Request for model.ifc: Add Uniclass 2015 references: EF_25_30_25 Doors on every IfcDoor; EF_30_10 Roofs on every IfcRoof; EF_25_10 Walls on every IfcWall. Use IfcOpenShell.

First a look at what the model holds.

```python
import ifcopenshell

model = ifcopenshell.open("model.ifc")
print(model.schema)
print("classifications:", [c.Name for c in model.by_type("IfcClassification")])
for ifc_class in ("IfcDoor", "IfcRoof", "IfcStair", "IfcWall", "IfcWindow"):
    print(ifc_class, len(model.by_type(ifc_class)))
```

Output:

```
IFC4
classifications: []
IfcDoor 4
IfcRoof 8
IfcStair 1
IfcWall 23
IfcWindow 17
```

```python
import ifcopenshell
import ifcopenshell.api.classification

model = ifcopenshell.open("model.ifc")

system = ifcopenshell.api.classification.add_classification(model, classification="Uniclass 2015")

codes = {
    "IfcDoor": ("EF_25_30_25", "Doors"),
    "IfcRoof": ("EF_30_10", "Roofs"),
    "IfcWall": ("EF_25_10", "Walls"),
}
for ifc_class, (code, name) in codes.items():
    products = model.by_type(ifc_class)
    ifcopenshell.api.classification.add_reference(
        model, products=products, classification=system, identification=code, name=name
    )
    print(code, len(products))

model.write("model_rev.ifc")
```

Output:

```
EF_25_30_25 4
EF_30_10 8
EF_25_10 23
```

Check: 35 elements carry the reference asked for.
